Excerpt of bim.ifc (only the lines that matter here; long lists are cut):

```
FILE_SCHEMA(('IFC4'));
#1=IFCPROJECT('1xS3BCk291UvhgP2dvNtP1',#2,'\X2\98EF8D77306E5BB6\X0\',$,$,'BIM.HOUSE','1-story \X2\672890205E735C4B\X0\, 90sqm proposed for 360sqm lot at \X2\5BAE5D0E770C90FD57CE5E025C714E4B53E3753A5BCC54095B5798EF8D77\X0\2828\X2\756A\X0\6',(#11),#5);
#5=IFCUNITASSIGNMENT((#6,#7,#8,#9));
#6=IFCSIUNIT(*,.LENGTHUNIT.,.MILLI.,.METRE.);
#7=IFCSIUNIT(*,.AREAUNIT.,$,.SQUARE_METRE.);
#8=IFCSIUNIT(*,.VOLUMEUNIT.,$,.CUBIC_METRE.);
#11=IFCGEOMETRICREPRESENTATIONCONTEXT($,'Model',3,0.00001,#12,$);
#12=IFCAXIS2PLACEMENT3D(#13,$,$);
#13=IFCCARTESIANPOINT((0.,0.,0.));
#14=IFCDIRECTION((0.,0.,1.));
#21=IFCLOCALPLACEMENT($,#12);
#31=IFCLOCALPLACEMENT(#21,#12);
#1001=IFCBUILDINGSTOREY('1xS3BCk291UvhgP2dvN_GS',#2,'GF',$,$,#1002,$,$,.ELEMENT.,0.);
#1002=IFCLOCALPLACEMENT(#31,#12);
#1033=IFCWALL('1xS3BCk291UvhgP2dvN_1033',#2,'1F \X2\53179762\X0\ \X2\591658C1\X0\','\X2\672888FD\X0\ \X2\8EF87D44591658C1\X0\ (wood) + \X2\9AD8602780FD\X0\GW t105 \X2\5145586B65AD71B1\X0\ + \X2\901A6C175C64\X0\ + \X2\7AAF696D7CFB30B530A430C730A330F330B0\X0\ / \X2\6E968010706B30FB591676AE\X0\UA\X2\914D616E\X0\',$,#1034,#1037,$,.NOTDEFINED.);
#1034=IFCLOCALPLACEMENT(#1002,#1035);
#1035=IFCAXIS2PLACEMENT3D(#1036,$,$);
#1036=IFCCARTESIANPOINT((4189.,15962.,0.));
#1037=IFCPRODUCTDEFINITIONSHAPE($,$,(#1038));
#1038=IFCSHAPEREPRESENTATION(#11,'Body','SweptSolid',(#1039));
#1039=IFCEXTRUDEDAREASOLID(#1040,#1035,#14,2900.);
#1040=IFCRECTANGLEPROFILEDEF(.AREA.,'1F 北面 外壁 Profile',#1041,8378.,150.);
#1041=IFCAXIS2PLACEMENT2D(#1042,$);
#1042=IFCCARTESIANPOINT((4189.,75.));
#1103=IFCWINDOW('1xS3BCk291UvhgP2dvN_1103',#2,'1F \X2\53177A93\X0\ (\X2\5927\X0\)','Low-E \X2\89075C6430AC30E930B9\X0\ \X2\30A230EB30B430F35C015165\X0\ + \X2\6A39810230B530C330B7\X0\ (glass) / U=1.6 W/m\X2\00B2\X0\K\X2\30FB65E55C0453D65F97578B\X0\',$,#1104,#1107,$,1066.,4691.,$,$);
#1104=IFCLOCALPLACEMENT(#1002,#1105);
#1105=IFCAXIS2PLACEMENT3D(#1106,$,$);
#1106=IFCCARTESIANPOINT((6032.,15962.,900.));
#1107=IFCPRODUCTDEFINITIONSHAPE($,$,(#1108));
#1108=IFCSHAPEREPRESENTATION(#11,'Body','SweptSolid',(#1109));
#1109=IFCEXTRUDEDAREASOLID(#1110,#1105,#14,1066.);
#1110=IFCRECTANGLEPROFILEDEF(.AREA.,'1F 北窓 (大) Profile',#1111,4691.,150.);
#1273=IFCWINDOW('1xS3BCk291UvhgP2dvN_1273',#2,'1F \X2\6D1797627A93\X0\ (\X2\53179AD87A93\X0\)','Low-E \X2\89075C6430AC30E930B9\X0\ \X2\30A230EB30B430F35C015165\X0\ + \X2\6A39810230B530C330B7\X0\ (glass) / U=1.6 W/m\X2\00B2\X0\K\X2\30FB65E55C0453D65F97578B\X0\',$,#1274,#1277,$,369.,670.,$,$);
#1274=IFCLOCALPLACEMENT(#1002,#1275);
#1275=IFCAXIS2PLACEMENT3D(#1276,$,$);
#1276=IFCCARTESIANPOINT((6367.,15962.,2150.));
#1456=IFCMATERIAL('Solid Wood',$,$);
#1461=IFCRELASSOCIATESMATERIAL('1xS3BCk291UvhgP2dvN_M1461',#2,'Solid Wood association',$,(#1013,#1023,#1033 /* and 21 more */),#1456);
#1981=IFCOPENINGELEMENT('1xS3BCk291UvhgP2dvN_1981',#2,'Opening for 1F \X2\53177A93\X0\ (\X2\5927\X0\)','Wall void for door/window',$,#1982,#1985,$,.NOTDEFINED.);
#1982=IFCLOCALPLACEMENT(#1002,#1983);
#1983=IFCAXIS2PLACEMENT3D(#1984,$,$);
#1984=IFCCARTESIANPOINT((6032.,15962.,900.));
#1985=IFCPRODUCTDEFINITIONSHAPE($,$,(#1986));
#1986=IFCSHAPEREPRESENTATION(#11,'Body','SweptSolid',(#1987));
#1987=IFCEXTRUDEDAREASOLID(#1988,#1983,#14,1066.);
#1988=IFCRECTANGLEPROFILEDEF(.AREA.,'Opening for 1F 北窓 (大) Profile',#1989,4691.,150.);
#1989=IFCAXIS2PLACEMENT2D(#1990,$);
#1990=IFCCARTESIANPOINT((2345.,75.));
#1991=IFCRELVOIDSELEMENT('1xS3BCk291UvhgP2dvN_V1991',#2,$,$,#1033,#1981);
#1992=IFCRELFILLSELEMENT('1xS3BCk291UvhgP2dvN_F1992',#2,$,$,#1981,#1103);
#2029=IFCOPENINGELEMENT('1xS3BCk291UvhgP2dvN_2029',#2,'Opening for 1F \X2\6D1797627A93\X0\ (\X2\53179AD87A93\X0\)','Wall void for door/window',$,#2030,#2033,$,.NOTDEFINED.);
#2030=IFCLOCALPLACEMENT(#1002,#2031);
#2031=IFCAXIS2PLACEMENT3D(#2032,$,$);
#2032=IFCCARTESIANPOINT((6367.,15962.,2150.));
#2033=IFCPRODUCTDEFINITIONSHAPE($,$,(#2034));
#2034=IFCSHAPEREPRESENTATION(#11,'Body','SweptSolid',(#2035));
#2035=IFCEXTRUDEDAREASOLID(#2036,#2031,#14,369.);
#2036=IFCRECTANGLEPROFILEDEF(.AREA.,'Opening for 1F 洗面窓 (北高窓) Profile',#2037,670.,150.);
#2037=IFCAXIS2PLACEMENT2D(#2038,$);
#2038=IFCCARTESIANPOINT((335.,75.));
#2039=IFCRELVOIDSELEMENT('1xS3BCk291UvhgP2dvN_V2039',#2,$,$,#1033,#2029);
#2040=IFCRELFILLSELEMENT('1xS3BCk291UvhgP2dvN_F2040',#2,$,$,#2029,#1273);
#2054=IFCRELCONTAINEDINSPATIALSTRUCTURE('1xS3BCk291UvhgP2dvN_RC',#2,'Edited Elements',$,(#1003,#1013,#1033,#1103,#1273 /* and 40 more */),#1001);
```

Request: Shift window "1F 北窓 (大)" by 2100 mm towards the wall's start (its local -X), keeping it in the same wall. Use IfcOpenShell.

```python
import ifcopenshell
import ifcopenshell.api.geometry
import ifcopenshell.util.placement

model = ifcopenshell.open("bim.ifc")

window = model.by_id(1103)
opening = window.FillsVoids[0].RelatingOpeningElement
wall = opening.VoidsElements[0].RelatingBuildingElement

wall_matrix = ifcopenshell.util.placement.get_local_placement(wall.ObjectPlacement)
shift = wall_matrix[:3, 0] * -2100.0
before = ifcopenshell.util.placement.get_local_placement(window.ObjectPlacement)[:3, 3].copy()

# The window is not placed relative to its opening, so move both.
for product in (opening, window):
    matrix = ifcopenshell.util.placement.get_local_placement(product.ObjectPlacement)
    matrix[:3, 3] += shift
    ifcopenshell.api.geometry.edit_object_placement(model, product=product, matrix=matrix, is_si=False)

after = ifcopenshell.util.placement.get_local_placement(window.ObjectPlacement)[:3, 3]
print("window moved by", (after - before).round(3) + 0.0)

model.write("bim_updated.ifc")
```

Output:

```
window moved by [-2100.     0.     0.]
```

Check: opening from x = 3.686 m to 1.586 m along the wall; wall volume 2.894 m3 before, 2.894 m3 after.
